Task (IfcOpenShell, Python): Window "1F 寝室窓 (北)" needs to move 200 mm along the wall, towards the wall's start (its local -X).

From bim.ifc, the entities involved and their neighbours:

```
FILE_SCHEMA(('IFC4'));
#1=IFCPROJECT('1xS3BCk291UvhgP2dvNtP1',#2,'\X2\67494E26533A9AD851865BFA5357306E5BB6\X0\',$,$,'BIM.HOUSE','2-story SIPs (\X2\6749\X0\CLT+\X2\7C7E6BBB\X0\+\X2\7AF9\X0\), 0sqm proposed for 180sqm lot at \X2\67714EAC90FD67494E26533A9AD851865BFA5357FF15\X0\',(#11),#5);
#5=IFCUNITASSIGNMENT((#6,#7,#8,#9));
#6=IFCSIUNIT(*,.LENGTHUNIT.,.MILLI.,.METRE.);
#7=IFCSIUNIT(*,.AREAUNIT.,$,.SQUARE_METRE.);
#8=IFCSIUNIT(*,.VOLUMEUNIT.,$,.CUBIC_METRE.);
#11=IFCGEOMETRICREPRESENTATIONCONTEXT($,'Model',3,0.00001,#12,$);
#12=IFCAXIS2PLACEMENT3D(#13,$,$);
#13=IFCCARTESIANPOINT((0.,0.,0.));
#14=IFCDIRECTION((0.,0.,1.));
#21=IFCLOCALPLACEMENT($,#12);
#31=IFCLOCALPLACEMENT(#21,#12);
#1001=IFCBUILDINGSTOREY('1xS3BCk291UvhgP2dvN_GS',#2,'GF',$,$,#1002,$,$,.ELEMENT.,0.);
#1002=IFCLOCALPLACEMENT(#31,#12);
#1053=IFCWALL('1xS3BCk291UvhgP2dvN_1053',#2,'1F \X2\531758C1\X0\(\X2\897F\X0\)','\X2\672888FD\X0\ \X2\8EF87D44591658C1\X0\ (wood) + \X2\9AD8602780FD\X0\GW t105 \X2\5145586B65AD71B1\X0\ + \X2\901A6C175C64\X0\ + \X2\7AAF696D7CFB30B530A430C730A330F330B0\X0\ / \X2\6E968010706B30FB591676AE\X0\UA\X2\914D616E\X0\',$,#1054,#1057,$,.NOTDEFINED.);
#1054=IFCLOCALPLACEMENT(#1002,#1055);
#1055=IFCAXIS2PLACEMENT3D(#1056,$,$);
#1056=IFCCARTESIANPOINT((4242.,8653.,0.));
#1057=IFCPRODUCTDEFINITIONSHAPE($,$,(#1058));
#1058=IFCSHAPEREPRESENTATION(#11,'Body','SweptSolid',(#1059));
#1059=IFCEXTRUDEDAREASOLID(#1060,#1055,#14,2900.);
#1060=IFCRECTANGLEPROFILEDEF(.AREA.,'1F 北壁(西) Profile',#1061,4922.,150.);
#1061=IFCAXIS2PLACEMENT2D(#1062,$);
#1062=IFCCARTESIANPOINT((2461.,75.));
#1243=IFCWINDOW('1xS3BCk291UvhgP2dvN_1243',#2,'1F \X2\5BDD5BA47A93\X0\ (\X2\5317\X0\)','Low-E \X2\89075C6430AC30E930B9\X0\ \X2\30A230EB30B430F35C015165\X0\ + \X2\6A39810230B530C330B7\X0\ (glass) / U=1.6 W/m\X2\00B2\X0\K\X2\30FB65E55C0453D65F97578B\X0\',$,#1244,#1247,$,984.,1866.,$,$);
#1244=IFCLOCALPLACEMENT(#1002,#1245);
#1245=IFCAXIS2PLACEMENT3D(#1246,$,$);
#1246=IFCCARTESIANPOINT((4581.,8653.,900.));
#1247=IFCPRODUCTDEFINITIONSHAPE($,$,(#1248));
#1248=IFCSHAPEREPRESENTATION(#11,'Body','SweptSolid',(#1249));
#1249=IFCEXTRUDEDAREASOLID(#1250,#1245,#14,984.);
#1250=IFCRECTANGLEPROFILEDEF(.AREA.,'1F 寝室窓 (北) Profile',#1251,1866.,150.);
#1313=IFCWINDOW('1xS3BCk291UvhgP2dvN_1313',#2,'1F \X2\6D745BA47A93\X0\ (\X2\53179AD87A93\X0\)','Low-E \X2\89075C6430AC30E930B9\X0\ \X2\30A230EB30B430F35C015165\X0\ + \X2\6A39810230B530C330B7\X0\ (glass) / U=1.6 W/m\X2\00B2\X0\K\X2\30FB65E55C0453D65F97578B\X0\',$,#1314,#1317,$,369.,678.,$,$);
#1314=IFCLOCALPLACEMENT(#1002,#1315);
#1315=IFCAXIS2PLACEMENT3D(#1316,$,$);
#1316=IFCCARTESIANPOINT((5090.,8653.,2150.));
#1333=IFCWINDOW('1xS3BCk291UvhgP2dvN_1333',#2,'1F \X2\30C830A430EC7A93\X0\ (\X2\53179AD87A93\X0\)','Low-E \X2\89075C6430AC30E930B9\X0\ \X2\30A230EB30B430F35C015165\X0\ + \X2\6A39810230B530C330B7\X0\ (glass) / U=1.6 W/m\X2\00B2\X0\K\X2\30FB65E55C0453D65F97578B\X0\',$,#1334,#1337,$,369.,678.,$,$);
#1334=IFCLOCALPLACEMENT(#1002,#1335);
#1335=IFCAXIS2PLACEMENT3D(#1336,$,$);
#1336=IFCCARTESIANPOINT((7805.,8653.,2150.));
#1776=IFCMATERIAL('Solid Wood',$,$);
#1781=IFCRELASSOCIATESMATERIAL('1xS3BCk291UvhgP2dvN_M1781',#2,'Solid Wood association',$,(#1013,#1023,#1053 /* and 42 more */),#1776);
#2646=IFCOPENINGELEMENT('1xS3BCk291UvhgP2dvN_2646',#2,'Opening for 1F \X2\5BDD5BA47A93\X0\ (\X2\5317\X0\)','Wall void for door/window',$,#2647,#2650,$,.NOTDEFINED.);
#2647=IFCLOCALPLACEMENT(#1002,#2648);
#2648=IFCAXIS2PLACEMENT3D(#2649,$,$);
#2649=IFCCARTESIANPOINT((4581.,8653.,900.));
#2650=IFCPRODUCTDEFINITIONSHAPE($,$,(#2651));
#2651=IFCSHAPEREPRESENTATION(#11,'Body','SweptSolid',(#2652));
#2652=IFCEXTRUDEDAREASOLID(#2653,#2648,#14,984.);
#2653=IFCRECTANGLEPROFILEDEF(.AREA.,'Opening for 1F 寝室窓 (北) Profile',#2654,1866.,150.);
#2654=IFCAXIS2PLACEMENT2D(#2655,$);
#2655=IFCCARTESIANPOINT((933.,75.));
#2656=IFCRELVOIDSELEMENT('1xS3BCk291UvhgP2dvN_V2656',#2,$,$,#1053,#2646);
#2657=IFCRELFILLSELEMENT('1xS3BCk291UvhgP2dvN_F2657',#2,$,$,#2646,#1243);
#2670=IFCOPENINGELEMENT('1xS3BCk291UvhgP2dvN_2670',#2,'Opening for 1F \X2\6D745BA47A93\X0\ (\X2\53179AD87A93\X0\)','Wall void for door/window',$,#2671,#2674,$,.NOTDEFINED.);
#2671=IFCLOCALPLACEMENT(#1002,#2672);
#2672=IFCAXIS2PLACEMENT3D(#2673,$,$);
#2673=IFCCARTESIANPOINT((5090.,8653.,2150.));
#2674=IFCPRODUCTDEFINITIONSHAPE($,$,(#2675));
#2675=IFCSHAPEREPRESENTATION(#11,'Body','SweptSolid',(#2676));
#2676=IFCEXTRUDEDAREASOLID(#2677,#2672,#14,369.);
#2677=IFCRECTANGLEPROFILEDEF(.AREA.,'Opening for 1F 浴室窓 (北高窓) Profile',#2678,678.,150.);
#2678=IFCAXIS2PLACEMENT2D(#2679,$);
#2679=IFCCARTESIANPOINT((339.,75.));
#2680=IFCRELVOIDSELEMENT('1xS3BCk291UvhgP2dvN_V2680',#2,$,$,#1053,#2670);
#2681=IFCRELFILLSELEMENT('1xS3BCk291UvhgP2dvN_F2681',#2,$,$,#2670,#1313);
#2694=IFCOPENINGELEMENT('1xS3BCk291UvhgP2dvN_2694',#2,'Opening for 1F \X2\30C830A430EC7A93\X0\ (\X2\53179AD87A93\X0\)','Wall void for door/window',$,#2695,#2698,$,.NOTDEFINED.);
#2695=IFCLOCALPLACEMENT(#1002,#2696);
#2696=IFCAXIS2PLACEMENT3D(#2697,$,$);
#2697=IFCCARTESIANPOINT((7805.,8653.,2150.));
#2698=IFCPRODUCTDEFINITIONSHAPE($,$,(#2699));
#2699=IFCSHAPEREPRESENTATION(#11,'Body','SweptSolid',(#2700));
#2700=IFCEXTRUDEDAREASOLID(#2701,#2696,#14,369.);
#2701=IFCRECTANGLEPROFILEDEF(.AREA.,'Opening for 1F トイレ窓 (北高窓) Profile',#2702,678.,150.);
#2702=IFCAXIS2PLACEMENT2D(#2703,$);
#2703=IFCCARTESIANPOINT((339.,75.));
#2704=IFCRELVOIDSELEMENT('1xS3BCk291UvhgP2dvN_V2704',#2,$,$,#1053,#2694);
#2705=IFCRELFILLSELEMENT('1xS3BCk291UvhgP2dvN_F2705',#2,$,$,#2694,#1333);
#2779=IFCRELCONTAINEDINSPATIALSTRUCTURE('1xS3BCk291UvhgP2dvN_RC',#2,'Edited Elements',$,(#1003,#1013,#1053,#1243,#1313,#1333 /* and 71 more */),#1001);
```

```python
import ifcopenshell
import ifcopenshell.api.geometry
import ifcopenshell.util.placement

model = ifcopenshell.open("bim.ifc")

window = model.by_id(1243)
opening = window.FillsVoids[0].RelatingOpeningElement
wall = opening.VoidsElements[0].RelatingBuildingElement

wall_matrix = ifcopenshell.util.placement.get_local_placement(wall.ObjectPlacement)
shift = wall_matrix[:3, 0] * -200.0
before = ifcopenshell.util.placement.get_local_placement(window.ObjectPlacement)[:3, 3].copy()

# The window is not placed relative to its opening, so move both.
for product in (opening, window):
    matrix = ifcopenshell.util.placement.get_local_placement(product.ObjectPlacement)
    matrix[:3, 3] += shift
    ifcopenshell.api.geometry.edit_object_placement(model, product=product, matrix=matrix, is_si=False)

after = ifcopenshell.util.placement.get_local_placement(window.ObjectPlacement)[:3, 3]
print("window moved by", (after - before).round(3) + 0.0)

model.write("bim_updated.ifc")
```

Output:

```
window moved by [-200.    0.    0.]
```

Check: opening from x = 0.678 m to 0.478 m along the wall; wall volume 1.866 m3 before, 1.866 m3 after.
